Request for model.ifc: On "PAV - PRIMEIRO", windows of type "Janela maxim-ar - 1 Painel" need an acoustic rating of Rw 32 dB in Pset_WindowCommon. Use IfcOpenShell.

First a look at what the model holds.

```python
import ifcopenshell
import ifcopenshell.util.element

model = ifcopenshell.open("model.ifc")
print(model.schema)
storey = next(s for s in model.by_type("IfcBuildingStorey") if s.Name == "PAV - PRIMEIRO")
windows = [e for e in ifcopenshell.util.element.get_decomposition(storey) if e.is_a("IfcWindow")]
seen = {}
for e in windows:
    element_type = ifcopenshell.util.element.get_type(e)
    key = (element_type.Name if element_type != e and element_type else None, ifcopenshell.util.element.get_pset(e, "Pset_WindowCommon", "AcousticRating"))
    seen[key] = seen.get(key, 0) + 1
for (name, value), count in sorted(seen.items(), key=str):
    print(count, "x", name, "|", value)
```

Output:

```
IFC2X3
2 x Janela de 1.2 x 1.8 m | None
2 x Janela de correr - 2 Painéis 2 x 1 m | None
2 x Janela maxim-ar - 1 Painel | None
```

```python
import ifcopenshell
import ifcopenshell.api.pset
import ifcopenshell.util.element

model = ifcopenshell.open("model.ifc")

storey = next(s for s in model.by_type("IfcBuildingStorey") if s.Name == "PAV - PRIMEIRO")
windows = [e for e in ifcopenshell.util.element.get_decomposition(storey) if e.is_a("IfcWindow")]

count = 0
for e in windows:
    element_type = ifcopenshell.util.element.get_type(e)
    if element_type in (None, e) or element_type.Name != "Janela maxim-ar - 1 Painel":
        continue
    # add_pset returns the element's existing set when there is one.
    pset = ifcopenshell.api.pset.add_pset(model, product=e, name="Pset_WindowCommon")
    ifcopenshell.api.pset.edit_pset(model, pset=pset, properties={"AcousticRating": "Rw 32 dB"})
    count += 1

print(count, "windows updated")

model.write("model-out.ifc")
```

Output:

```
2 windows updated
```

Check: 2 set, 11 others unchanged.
